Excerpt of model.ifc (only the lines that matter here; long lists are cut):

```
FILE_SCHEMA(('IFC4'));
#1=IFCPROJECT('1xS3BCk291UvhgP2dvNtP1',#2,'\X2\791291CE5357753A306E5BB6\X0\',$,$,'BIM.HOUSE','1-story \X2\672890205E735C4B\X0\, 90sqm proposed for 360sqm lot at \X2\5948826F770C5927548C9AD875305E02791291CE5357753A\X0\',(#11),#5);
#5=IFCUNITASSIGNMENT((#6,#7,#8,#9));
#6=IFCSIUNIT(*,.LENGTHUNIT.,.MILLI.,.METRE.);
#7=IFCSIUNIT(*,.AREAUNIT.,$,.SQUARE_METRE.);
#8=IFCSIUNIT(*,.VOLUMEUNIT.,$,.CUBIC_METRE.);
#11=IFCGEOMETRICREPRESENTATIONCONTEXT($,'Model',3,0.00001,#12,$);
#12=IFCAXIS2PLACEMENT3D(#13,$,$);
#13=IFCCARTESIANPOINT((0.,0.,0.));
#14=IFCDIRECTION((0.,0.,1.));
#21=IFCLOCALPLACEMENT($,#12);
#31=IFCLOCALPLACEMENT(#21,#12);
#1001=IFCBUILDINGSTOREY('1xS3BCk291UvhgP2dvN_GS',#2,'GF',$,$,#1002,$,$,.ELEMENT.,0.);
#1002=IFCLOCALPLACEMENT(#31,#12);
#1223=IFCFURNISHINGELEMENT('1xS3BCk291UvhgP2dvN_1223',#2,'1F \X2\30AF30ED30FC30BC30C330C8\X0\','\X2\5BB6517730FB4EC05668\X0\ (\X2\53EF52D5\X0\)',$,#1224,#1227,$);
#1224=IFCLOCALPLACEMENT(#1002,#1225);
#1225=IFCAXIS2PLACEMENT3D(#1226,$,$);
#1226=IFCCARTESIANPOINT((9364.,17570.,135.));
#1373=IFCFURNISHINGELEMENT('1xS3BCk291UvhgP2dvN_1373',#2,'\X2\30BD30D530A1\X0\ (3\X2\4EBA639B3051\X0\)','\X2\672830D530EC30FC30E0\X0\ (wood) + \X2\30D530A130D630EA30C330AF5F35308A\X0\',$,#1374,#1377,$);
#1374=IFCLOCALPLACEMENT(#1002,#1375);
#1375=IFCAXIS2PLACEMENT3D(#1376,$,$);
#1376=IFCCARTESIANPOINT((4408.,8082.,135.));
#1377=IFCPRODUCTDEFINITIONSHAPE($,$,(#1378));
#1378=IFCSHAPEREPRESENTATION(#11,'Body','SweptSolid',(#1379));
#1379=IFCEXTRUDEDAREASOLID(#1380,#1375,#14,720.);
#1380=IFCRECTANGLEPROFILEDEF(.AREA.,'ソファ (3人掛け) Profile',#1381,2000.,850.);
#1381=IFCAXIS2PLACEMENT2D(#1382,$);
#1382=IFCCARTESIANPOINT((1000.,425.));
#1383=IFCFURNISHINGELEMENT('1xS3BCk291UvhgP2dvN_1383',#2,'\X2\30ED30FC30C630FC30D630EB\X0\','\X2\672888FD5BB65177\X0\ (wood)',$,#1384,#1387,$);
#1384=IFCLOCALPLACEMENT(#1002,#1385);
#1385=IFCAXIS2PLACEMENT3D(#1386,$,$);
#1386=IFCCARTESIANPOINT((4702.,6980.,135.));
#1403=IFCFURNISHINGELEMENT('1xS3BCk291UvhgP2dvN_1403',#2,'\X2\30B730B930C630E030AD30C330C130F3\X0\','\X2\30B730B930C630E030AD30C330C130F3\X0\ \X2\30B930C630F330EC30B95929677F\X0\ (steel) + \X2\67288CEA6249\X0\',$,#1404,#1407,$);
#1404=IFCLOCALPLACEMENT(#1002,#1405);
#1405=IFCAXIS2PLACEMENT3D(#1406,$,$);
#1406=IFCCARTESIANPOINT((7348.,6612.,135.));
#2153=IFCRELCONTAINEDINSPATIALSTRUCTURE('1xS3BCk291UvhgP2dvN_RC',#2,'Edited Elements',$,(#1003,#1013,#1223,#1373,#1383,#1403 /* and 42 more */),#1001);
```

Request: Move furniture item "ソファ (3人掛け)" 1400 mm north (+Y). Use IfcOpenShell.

```python
import ifcopenshell
import ifcopenshell.api.geometry
import ifcopenshell.util.placement
import ifcopenshell.util.unit

model = ifcopenshell.open("model.ifc")
unit_scale = ifcopenshell.util.unit.calculate_unit_scale(model)

item = model.by_guid("1xS3BCk291UvhgP2dvN_1373")
matrix = ifcopenshell.util.placement.get_local_placement(item.ObjectPlacement)
matrix[1, 3] += 1.4 / unit_scale
ifcopenshell.api.geometry.edit_object_placement(model, product=item, matrix=matrix, is_si=False)

print(ifcopenshell.util.placement.get_local_placement(item.ObjectPlacement).round(3) + 0.0)

model.write("model_edited.ifc")
```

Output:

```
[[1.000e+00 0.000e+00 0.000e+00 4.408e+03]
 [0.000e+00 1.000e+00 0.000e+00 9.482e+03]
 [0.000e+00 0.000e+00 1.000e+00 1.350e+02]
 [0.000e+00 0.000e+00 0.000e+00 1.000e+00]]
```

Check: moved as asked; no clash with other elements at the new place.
